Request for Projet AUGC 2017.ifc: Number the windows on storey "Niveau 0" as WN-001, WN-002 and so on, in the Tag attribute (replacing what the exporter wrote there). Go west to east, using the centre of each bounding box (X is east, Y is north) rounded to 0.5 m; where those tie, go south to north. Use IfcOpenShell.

First a look at what the model holds.

```python
import ifcopenshell
import ifcopenshell.util.element
import ifcopenshell.util.placement

model = ifcopenshell.open("Projet AUGC 2017.ifc")
print(model.schema)
storey = next(s for s in model.by_type("IfcBuildingStorey") if s.Name == "Niveau 0")
windows = [e for e in ifcopenshell.util.element.get_decomposition(storey) if e.is_a("IfcWindow")]
for e in sorted(windows, key=lambda e: e.id()):
    origin = ifcopenshell.util.placement.get_local_placement(e.ObjectPlacement)[:3, 3]
    print(e.id(), e.Tag, e.Name, origin.round(2) + 0.0, sep=" | ")
```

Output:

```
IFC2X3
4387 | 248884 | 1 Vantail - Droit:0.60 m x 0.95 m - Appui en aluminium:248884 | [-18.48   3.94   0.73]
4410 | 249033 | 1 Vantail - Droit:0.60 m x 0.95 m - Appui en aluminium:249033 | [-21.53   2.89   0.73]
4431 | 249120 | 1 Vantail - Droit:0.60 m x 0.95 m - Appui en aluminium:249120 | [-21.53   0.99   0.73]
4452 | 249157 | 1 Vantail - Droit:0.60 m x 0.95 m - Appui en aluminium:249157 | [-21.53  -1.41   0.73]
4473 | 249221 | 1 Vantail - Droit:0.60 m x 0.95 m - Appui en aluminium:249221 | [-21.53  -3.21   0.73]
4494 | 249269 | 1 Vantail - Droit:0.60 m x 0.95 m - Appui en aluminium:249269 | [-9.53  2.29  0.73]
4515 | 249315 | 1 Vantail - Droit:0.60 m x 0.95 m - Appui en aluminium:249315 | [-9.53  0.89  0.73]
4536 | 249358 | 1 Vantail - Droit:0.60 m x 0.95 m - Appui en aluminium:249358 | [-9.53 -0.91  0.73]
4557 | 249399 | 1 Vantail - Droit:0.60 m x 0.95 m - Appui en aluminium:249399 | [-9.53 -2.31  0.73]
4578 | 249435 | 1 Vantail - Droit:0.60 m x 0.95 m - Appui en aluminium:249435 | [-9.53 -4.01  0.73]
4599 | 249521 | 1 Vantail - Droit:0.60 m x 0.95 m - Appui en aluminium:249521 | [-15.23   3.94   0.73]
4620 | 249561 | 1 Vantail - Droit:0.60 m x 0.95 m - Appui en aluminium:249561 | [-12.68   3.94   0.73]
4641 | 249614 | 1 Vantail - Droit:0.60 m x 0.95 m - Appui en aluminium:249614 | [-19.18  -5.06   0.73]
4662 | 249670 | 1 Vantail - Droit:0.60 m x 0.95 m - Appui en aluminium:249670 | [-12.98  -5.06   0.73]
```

```python
import ifcopenshell
import ifcopenshell.geom
import ifcopenshell.util.element
import ifcopenshell.util.shape

model = ifcopenshell.open("Projet AUGC 2017.ifc")
settings = ifcopenshell.geom.settings()
settings.set("use-world-coords", True)


def centre(element):
    shape = ifcopenshell.geom.create_shape(settings, element)
    return ifcopenshell.util.shape.get_bbox_centroid(shape.geometry)


storey = next(s for s in model.by_type("IfcBuildingStorey") if s.Name == "Niveau 0")
windows = [e for e in ifcopenshell.util.element.get_decomposition(storey) if e.is_a("IfcWindow")]

# Insertion points can sit at a corner or the storey origin, so sort by the geometry (in metres).
centres = {e: centre(e) for e in windows}
windows.sort(key=lambda e: (round(centres[e][0] / 0.5), centres[e][1]))

for i, e in enumerate(windows, start=1):
    number = f"WN-0{i:02d}"
    e.Tag = number
    print(e.id(), number)

model.write("Projet AUGC 2017_edited.ifc")
```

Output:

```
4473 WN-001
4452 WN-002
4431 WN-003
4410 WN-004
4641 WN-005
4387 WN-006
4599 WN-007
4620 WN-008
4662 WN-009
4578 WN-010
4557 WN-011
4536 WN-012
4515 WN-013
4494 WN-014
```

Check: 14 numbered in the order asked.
